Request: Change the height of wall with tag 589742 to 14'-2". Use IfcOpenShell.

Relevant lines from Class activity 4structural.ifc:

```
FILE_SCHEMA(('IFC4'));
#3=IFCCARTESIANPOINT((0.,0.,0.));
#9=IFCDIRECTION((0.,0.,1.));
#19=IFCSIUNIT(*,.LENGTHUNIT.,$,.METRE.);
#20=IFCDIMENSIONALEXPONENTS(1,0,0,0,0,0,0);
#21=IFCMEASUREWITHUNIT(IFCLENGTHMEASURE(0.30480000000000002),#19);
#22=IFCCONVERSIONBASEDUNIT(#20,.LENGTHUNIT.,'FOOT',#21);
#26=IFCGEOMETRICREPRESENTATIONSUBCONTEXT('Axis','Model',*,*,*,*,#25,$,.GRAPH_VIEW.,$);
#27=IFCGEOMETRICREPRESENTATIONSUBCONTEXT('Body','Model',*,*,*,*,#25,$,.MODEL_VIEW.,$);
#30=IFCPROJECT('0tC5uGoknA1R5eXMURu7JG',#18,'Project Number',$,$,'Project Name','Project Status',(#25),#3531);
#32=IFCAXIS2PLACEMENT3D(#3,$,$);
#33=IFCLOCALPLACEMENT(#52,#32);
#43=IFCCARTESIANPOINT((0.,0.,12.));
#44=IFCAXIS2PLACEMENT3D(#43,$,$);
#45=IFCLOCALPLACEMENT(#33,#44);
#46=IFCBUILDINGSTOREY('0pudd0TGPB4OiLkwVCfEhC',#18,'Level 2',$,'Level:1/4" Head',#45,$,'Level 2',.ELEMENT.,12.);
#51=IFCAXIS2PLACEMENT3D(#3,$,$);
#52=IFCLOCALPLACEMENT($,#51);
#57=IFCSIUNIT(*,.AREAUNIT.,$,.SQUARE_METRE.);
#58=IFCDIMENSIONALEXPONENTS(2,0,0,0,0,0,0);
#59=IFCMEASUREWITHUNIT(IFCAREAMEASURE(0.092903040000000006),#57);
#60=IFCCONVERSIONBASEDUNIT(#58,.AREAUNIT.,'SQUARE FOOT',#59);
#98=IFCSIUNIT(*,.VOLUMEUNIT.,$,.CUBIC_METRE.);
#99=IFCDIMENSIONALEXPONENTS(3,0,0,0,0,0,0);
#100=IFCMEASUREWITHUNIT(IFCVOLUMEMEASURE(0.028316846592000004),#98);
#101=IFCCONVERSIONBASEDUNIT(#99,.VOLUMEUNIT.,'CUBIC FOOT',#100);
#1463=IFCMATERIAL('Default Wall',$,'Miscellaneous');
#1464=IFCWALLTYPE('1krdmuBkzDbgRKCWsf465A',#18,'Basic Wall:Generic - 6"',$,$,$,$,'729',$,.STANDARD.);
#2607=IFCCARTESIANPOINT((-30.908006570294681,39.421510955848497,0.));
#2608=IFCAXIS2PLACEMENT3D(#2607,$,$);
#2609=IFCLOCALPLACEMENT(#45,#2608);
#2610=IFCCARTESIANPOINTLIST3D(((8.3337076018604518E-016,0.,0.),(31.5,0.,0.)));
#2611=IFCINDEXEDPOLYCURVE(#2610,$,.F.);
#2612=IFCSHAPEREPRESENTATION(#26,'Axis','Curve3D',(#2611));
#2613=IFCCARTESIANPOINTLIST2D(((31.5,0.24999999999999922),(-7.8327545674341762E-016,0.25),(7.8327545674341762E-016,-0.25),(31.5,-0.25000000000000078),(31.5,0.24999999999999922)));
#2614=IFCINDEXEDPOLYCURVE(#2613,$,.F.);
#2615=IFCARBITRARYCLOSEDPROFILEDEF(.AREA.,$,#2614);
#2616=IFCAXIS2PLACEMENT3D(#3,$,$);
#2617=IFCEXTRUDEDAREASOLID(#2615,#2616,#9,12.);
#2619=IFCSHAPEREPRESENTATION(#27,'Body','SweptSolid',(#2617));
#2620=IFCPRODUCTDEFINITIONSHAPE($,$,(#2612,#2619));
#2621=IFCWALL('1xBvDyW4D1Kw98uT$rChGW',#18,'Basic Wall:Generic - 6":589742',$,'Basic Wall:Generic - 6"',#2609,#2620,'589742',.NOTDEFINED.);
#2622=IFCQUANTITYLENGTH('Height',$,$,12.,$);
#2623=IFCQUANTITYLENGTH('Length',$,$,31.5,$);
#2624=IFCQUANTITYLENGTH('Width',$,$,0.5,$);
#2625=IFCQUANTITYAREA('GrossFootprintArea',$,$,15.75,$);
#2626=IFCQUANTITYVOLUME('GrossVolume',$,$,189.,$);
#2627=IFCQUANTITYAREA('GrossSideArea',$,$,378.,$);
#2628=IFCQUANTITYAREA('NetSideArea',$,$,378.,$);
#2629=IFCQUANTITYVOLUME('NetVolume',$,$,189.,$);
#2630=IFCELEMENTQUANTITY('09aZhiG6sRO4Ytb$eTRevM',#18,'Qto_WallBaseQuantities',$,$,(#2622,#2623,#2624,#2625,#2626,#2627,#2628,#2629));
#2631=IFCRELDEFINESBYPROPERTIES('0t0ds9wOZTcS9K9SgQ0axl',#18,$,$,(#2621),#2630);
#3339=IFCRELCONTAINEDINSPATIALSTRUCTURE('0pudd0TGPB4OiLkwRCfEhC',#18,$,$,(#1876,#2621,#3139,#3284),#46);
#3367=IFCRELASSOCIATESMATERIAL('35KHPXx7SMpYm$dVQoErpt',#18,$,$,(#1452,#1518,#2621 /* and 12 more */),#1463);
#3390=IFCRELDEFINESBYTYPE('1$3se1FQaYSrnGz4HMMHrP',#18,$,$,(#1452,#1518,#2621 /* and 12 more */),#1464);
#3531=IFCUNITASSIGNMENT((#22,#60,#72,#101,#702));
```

```python
import ifcopenshell
import ifcopenshell.api.pset
import ifcopenshell.geom
import ifcopenshell.util.element
import ifcopenshell.util.representation
import ifcopenshell.util.shape
import ifcopenshell.util.unit

model = ifcopenshell.open("Class activity 4structural.ifc")
unit_scale = ifcopenshell.util.unit.calculate_unit_scale(model)
area_scale = ifcopenshell.util.unit.calculate_unit_scale(model, "AREAUNIT")
volume_scale = ifcopenshell.util.unit.calculate_unit_scale(model, "VOLUMEUNIT")
settings = ifcopenshell.geom.settings()


def volume(element):
    """Net volume in cubic metres, openings subtracted."""
    shape = ifcopenshell.geom.create_shape(settings, element)
    return ifcopenshell.util.shape.get_volume(shape.geometry)


wall = model.by_guid("1xBvDyW4D1Kw98uT$rChGW")
before = volume(wall)

body = ifcopenshell.util.representation.get_representation(wall, "Model", "Body")
solid = body.Items[0]
old_height = solid.Depth
solid.Depth = 170 * 0.0254 / unit_scale
after = volume(wall)
thickness = 0.1524  # wall thickness in metres

# Update the stored height, areas and volumes.
qto = model.by_id(ifcopenshell.util.element.get_pset(wall, "Qto_WallBaseQuantities", should_inherit=False)["id"])
ifcopenshell.api.pset.edit_qto(model, qto=qto, properties={
    "Height": solid.Depth,
    "GrossVolume": ifcopenshell.util.element.get_pset(wall, "Qto_WallBaseQuantities", "GrossVolume") * solid.Depth / old_height,
    "GrossSideArea": ifcopenshell.util.element.get_pset(wall, "Qto_WallBaseQuantities", "GrossSideArea") * solid.Depth / old_height,
    "NetSideArea": after / thickness / area_scale,
    "NetVolume": after / volume_scale,
})

print(f"height {old_height:g} -> {solid.Depth:g}, volume {before:.3f} -> {after:.3f} m3")

model.write("Class activity 4structural_updated.ifc")
```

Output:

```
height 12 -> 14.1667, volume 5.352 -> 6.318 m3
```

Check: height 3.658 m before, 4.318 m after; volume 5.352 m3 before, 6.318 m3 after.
